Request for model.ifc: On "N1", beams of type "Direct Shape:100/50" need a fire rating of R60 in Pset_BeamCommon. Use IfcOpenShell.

First a look at what the model holds.

```python
import ifcopenshell
import ifcopenshell.util.element

model = ifcopenshell.open("model.ifc")
print(model.schema)
storey = next(s for s in model.by_type("IfcBuildingStorey") if s.Name == "N1")
beams = [e for e in ifcopenshell.util.element.get_decomposition(storey) if e.is_a("IfcBeam")]
seen = {}
for e in beams:
    element_type = ifcopenshell.util.element.get_type(e)
    key = (element_type.Name if element_type != e and element_type else None, ifcopenshell.util.element.get_pset(e, "Pset_BeamCommon", "FireRating"))
    seen[key] = seen.get(key, 0) + 1
for (name, value), count in sorted(seen.items(), key=str):
    print(count, "x", name, "|", value)
```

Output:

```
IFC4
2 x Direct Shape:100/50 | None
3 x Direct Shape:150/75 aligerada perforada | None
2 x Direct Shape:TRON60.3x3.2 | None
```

```python
import ifcopenshell
import ifcopenshell.api.pset
import ifcopenshell.util.element

model = ifcopenshell.open("model.ifc")

storey = next(s for s in model.by_type("IfcBuildingStorey") if s.Name == "N1")
beams = [e for e in ifcopenshell.util.element.get_decomposition(storey) if e.is_a("IfcBeam")]

count = 0
for e in beams:
    element_type = ifcopenshell.util.element.get_type(e)
    if element_type in (None, e) or element_type.Name != "Direct Shape:100/50":
        continue
    # add_pset returns the element's existing set when there is one.
    pset = ifcopenshell.api.pset.add_pset(model, product=e, name="Pset_BeamCommon")
    ifcopenshell.api.pset.edit_pset(model, pset=pset, properties={"FireRating": "R60"})
    count += 1

print(count, "beams updated")

model.write("model_updated.ifc")
```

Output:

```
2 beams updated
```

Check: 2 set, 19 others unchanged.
